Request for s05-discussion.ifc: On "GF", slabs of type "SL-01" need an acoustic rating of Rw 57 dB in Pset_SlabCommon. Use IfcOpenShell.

First a look at what the model holds.

```python
import ifcopenshell
import ifcopenshell.util.element

model = ifcopenshell.open("s05-discussion.ifc")
print(model.schema)
storey = next(s for s in model.by_type("IfcBuildingStorey") if s.Name == "GF")
slabs = [e for e in ifcopenshell.util.element.get_decomposition(storey) if e.is_a("IfcSlab")]
seen = {}
for e in slabs:
    element_type = ifcopenshell.util.element.get_type(e)
    key = (element_type.Name if element_type != e and element_type else None, ifcopenshell.util.element.get_pset(e, "Pset_SlabCommon", "AcousticRating"))
    seen[key] = seen.get(key, 0) + 1
for (name, value), count in sorted(seen.items(), key=str):
    print(count, "x", name, "|", value)
```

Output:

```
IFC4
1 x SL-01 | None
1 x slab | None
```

```python
import ifcopenshell
import ifcopenshell.api.pset
import ifcopenshell.util.element

model = ifcopenshell.open("s05-discussion.ifc")

storey = next(s for s in model.by_type("IfcBuildingStorey") if s.Name == "GF")
slabs = [e for e in ifcopenshell.util.element.get_decomposition(storey) if e.is_a("IfcSlab")]

count = 0
for e in slabs:
    element_type = ifcopenshell.util.element.get_type(e)
    if element_type in (None, e) or element_type.Name != "SL-01":
        continue
    # add_pset returns the element's existing set when there is one.
    pset = ifcopenshell.api.pset.add_pset(model, product=e, name="Pset_SlabCommon")
    ifcopenshell.api.pset.edit_pset(model, pset=pset, properties={"AcousticRating": "Rw 57 dB"})
    count += 1

print(count, "slabs updated")

model.write("s05-discussion_rev.ifc")
```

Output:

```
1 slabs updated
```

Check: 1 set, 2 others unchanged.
